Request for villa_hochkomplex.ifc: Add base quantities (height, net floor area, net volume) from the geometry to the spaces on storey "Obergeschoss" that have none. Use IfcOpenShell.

First a look at what the model holds.

```python
import ifcopenshell
import ifcopenshell.util.element
import ifcopenshell.util.unit

model = ifcopenshell.open("villa_hochkomplex.ifc")
print(model.schema)
for unit_type in ("LENGTHUNIT", "AREAUNIT", "VOLUMEUNIT"):
    print(unit_type, ifcopenshell.util.unit.calculate_unit_scale(model, unit_type))
storey = next(s for s in model.by_type("IfcBuildingStorey") if s.Name == "Obergeschoss")
spaces = [e for e in ifcopenshell.util.element.get_decomposition(storey) if e.is_a("IfcSpace")]
for e in sorted(spaces, key=lambda e: e.id()):
    print(e.id(), e.is_a(), e.Name, list(ifcopenshell.util.element.get_psets(e, qtos_only=True)), sep=" | ")
```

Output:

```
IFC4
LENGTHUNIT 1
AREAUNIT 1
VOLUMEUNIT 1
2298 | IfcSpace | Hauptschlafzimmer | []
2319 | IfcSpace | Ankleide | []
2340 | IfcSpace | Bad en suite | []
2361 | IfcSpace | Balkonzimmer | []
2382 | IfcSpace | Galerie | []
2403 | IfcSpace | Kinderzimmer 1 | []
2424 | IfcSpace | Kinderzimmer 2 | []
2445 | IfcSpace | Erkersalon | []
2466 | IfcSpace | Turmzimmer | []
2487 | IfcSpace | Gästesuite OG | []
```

```python
import ifcopenshell
import ifcopenshell.api.pset
import ifcopenshell.geom
import ifcopenshell.util.element
import ifcopenshell.util.shape
import ifcopenshell.util.unit

model = ifcopenshell.open("villa_hochkomplex.ifc")
unit_scale = ifcopenshell.util.unit.calculate_unit_scale(model)
area_scale = ifcopenshell.util.unit.calculate_unit_scale(model, "AREAUNIT")
volume_scale = ifcopenshell.util.unit.calculate_unit_scale(model, "VOLUMEUNIT")
settings = ifcopenshell.geom.settings()

storey = next(s for s in model.by_type("IfcBuildingStorey") if s.Name == "Obergeschoss")
spaces = [e for e in ifcopenshell.util.element.get_decomposition(storey) if e.is_a("IfcSpace")]

for e in sorted(spaces, key=lambda e: e.id()):
    if ifcopenshell.util.element.get_psets(e, qtos_only=True, should_inherit=False):
        continue
    # Geometry comes back in metres, in the element's own axes.
    shape = ifcopenshell.geom.create_shape(settings, e)
    values = {
        "Height": ifcopenshell.util.shape.get_z(shape.geometry) / unit_scale,
        "NetFloorArea": ifcopenshell.util.shape.get_footprint_area(shape.geometry) / area_scale,
        "NetVolume": ifcopenshell.util.shape.get_volume(shape.geometry) / volume_scale,
    }
    qto = ifcopenshell.api.pset.add_qto(model, product=e, name="Qto_SpaceBaseQuantities")
    ifcopenshell.api.pset.edit_qto(model, qto=qto, properties=values)
    print(e.id(), {k: round(v, 3) for k, v in values.items()})

model.write("villa_hochkomplex_updated.ifc")
```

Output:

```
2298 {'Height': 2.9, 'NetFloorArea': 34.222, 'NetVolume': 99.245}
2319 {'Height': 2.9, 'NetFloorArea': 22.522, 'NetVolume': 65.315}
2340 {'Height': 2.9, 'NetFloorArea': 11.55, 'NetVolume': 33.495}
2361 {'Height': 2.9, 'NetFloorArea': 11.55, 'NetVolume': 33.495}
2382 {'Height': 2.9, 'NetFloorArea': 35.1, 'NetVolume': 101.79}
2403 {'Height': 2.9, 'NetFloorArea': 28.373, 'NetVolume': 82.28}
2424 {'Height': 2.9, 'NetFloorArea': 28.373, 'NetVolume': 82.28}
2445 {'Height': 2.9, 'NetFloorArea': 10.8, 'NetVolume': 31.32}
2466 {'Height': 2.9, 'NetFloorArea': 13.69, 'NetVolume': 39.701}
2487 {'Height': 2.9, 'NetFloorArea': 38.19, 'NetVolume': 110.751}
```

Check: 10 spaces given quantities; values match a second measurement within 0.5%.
